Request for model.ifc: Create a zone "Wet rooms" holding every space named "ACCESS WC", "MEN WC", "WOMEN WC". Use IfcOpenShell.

First a look at what the model holds.

```python
import ifcopenshell

model = ifcopenshell.open("model.ifc")
print(model.schema)
seen = {}
for space in model.by_type("IfcSpace"):
    seen[space.LongName] = seen.get(space.LongName, 0) + 1
for name, count in sorted(seen.items(), key=str):
    print(count, "x", name)
print("zones:", [z.Name for z in model.by_type("IfcZone")][:20])
```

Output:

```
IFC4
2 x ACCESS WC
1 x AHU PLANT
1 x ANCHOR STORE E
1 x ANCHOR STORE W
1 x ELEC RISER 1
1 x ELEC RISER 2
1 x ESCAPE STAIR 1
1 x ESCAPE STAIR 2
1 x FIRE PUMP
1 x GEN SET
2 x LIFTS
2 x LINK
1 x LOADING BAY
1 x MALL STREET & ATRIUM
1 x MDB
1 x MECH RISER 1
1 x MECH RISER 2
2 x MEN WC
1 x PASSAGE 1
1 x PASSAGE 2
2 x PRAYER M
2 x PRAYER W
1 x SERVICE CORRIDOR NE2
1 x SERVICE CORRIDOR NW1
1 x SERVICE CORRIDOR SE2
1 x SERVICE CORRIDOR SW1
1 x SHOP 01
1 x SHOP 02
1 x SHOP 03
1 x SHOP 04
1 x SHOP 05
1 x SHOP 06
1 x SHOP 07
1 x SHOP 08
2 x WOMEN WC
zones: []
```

```python
import ifcopenshell
import ifcopenshell.api.group
import ifcopenshell.api.root

model = ifcopenshell.open("model.ifc")

names = {"ACCESS WC", "MEN WC", "WOMEN WC"}
spaces = [s for s in model.by_type("IfcSpace") if s.LongName in names]

zone = ifcopenshell.api.root.create_entity(model, ifc_class="IfcZone", name="Wet rooms")
ifcopenshell.api.group.assign_group(model, products=spaces, group=zone)
print(len(spaces), "spaces in", zone.Name)

model.write("model_rev.ifc")
```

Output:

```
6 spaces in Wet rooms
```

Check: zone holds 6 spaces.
